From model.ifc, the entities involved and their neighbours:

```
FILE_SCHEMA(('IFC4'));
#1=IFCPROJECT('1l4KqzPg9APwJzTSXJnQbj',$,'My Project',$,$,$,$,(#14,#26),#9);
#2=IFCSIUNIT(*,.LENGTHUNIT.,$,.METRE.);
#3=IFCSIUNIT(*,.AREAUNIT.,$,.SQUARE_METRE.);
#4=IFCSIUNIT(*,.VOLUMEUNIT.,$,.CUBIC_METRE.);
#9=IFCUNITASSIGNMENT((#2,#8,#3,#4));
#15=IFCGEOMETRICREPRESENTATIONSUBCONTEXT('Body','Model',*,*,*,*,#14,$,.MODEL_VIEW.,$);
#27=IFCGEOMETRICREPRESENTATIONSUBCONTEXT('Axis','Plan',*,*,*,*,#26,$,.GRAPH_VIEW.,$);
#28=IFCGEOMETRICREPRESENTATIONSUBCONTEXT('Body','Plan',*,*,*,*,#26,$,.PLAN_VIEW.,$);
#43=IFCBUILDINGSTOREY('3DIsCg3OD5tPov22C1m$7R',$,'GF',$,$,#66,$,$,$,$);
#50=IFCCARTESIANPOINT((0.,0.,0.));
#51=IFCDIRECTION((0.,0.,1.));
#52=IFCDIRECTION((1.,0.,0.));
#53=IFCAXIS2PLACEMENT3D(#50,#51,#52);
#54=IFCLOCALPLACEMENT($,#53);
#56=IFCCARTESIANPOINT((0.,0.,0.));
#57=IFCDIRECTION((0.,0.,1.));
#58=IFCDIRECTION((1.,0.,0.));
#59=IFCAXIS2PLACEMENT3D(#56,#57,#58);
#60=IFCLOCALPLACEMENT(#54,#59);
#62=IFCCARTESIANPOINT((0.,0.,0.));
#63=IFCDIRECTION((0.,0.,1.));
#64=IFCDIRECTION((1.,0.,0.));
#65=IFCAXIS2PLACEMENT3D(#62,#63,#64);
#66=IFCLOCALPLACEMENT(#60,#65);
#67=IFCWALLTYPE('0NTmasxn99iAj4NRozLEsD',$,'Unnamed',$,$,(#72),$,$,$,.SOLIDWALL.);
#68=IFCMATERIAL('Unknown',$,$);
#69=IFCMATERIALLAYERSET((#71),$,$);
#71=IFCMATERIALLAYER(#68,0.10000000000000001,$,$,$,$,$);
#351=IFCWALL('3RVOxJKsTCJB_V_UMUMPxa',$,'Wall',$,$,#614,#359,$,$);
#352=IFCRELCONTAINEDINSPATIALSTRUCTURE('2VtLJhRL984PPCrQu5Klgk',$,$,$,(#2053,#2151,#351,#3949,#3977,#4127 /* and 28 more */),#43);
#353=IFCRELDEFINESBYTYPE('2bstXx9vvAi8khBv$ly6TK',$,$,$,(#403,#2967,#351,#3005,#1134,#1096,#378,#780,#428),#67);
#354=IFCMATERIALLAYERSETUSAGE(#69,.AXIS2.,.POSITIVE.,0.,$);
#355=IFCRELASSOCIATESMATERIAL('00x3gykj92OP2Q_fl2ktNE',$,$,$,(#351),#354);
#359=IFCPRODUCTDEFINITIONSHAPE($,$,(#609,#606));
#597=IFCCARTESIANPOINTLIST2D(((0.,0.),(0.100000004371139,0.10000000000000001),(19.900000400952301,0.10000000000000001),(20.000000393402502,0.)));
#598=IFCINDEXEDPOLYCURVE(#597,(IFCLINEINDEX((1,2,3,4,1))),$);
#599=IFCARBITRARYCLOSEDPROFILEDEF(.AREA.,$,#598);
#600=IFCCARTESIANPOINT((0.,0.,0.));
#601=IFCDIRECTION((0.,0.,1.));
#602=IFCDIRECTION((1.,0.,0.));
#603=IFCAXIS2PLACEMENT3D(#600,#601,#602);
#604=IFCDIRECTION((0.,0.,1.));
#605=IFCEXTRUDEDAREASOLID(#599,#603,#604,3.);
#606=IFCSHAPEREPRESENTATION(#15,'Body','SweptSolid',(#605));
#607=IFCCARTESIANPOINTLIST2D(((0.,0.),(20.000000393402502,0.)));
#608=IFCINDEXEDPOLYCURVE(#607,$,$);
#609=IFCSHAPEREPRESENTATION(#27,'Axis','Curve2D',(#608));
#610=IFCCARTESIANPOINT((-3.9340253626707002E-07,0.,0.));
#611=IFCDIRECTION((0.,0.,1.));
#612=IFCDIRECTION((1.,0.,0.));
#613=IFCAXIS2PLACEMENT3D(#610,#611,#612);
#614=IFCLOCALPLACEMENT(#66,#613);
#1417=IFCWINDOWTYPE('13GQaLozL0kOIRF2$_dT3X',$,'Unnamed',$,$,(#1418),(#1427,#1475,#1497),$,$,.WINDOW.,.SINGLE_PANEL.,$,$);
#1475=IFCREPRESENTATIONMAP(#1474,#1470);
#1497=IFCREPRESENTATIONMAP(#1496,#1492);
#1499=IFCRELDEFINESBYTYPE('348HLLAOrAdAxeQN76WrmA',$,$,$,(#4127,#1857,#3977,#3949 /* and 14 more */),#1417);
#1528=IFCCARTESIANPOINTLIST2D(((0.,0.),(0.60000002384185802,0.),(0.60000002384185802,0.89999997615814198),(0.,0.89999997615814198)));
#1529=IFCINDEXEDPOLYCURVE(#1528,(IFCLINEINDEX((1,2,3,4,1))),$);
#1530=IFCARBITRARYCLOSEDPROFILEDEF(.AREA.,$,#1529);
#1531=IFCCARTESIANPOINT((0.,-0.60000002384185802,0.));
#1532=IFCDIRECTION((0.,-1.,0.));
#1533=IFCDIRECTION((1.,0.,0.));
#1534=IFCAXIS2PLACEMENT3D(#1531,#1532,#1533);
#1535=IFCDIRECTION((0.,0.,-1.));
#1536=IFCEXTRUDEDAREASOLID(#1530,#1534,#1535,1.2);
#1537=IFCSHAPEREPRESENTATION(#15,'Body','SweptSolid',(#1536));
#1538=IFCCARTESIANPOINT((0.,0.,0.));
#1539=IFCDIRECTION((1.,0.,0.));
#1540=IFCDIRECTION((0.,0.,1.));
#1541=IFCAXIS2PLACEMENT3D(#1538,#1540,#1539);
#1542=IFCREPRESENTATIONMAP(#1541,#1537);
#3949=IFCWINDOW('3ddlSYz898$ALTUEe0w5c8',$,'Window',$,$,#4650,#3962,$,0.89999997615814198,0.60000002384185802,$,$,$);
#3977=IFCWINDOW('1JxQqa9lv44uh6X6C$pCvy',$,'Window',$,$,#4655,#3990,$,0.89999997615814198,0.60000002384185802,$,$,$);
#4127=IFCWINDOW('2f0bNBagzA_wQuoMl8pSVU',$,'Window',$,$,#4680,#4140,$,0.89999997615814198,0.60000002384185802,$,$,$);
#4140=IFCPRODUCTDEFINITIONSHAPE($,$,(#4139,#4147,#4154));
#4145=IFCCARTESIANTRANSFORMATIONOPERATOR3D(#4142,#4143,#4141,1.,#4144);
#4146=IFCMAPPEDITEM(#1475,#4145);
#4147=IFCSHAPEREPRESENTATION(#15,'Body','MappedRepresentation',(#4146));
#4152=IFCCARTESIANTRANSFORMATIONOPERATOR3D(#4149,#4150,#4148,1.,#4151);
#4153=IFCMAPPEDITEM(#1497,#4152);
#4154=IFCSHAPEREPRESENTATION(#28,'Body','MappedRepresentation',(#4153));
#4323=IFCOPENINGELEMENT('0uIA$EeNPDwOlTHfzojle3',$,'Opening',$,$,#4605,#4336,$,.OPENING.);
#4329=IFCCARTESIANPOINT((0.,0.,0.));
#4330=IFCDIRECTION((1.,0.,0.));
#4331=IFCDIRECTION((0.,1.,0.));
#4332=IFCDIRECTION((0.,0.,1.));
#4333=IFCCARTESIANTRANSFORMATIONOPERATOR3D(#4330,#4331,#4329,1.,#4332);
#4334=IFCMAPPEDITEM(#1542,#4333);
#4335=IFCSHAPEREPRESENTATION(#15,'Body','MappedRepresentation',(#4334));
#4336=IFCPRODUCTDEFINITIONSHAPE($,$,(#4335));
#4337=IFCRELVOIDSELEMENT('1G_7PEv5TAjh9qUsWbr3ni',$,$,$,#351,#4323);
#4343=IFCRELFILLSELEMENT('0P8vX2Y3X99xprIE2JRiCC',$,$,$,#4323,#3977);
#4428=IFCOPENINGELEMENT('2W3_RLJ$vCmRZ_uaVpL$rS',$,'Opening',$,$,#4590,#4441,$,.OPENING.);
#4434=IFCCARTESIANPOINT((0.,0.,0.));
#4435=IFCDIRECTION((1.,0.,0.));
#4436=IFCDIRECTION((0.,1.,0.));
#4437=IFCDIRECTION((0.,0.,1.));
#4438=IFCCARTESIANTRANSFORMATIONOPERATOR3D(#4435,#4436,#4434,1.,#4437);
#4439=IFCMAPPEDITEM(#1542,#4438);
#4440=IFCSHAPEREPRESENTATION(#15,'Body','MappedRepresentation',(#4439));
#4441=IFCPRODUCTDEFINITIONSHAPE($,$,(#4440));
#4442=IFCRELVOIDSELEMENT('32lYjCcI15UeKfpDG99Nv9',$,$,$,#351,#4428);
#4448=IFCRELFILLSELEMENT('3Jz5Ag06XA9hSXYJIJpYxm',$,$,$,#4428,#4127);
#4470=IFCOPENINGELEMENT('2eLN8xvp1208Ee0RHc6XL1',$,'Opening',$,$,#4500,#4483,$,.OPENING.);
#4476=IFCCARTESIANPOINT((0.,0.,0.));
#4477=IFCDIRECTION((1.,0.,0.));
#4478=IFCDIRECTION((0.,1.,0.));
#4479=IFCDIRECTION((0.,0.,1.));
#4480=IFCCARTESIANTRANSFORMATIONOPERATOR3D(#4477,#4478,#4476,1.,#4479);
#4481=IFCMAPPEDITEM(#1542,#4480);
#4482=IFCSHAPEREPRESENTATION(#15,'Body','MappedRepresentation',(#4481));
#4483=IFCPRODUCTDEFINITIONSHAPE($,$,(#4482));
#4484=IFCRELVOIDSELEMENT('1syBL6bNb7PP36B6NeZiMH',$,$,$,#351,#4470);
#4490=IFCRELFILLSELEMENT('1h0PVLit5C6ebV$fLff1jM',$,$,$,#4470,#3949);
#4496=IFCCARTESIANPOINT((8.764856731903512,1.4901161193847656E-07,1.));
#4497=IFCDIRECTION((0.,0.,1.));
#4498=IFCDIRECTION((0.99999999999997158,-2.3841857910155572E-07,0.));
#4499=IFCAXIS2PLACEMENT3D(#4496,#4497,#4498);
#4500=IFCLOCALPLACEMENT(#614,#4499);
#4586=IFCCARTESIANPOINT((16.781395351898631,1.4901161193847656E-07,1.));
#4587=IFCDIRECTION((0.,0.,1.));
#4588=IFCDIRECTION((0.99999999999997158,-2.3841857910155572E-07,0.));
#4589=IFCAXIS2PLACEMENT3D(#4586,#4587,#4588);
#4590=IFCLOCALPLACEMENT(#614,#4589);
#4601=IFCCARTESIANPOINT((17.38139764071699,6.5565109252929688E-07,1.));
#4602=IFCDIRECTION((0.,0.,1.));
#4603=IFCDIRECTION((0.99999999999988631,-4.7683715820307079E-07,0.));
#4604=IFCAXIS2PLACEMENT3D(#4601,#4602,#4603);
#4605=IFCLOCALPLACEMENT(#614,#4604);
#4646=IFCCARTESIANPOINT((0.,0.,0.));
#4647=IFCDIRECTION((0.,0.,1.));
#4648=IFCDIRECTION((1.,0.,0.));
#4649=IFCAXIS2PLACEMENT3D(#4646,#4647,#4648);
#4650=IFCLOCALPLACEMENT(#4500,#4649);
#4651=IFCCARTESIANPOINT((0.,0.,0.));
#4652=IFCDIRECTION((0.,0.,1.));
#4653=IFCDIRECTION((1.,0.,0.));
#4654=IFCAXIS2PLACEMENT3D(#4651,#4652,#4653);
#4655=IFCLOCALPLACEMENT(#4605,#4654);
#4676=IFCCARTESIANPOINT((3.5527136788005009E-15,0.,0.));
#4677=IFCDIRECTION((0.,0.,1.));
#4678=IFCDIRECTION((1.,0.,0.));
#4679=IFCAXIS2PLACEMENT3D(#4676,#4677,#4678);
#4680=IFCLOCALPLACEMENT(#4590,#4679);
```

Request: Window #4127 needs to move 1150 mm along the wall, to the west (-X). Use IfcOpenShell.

```python
import ifcopenshell
import ifcopenshell.api.geometry
import ifcopenshell.util.placement
import ifcopenshell.util.unit

model = ifcopenshell.open("model.ifc")
unit_scale = ifcopenshell.util.unit.calculate_unit_scale(model)

window = model.by_guid("2f0bNBagzA_wQuoMl8pSVU")
opening = window.FillsVoids[0].RelatingOpeningElement
wall = opening.VoidsElements[0].RelatingBuildingElement

wall_matrix = ifcopenshell.util.placement.get_local_placement(wall.ObjectPlacement)
shift = wall_matrix[:3, 0] * -1.15 / unit_scale
before = ifcopenshell.util.placement.get_local_placement(window.ObjectPlacement)[:3, 3].copy()

# The window is placed relative to its opening, so it follows when the opening moves.
matrix = ifcopenshell.util.placement.get_local_placement(opening.ObjectPlacement)
matrix[:3, 3] += shift
ifcopenshell.api.geometry.edit_object_placement(
    model, product=opening, matrix=matrix, is_si=False, should_transform_children=True
)

after = ifcopenshell.util.placement.get_local_placement(window.ObjectPlacement)[:3, 3]
print("window moved by", (after - before).round(3) + 0.0)

model.write("model-out.ifc")
```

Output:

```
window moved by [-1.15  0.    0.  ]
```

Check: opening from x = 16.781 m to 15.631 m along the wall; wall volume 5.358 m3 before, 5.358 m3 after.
